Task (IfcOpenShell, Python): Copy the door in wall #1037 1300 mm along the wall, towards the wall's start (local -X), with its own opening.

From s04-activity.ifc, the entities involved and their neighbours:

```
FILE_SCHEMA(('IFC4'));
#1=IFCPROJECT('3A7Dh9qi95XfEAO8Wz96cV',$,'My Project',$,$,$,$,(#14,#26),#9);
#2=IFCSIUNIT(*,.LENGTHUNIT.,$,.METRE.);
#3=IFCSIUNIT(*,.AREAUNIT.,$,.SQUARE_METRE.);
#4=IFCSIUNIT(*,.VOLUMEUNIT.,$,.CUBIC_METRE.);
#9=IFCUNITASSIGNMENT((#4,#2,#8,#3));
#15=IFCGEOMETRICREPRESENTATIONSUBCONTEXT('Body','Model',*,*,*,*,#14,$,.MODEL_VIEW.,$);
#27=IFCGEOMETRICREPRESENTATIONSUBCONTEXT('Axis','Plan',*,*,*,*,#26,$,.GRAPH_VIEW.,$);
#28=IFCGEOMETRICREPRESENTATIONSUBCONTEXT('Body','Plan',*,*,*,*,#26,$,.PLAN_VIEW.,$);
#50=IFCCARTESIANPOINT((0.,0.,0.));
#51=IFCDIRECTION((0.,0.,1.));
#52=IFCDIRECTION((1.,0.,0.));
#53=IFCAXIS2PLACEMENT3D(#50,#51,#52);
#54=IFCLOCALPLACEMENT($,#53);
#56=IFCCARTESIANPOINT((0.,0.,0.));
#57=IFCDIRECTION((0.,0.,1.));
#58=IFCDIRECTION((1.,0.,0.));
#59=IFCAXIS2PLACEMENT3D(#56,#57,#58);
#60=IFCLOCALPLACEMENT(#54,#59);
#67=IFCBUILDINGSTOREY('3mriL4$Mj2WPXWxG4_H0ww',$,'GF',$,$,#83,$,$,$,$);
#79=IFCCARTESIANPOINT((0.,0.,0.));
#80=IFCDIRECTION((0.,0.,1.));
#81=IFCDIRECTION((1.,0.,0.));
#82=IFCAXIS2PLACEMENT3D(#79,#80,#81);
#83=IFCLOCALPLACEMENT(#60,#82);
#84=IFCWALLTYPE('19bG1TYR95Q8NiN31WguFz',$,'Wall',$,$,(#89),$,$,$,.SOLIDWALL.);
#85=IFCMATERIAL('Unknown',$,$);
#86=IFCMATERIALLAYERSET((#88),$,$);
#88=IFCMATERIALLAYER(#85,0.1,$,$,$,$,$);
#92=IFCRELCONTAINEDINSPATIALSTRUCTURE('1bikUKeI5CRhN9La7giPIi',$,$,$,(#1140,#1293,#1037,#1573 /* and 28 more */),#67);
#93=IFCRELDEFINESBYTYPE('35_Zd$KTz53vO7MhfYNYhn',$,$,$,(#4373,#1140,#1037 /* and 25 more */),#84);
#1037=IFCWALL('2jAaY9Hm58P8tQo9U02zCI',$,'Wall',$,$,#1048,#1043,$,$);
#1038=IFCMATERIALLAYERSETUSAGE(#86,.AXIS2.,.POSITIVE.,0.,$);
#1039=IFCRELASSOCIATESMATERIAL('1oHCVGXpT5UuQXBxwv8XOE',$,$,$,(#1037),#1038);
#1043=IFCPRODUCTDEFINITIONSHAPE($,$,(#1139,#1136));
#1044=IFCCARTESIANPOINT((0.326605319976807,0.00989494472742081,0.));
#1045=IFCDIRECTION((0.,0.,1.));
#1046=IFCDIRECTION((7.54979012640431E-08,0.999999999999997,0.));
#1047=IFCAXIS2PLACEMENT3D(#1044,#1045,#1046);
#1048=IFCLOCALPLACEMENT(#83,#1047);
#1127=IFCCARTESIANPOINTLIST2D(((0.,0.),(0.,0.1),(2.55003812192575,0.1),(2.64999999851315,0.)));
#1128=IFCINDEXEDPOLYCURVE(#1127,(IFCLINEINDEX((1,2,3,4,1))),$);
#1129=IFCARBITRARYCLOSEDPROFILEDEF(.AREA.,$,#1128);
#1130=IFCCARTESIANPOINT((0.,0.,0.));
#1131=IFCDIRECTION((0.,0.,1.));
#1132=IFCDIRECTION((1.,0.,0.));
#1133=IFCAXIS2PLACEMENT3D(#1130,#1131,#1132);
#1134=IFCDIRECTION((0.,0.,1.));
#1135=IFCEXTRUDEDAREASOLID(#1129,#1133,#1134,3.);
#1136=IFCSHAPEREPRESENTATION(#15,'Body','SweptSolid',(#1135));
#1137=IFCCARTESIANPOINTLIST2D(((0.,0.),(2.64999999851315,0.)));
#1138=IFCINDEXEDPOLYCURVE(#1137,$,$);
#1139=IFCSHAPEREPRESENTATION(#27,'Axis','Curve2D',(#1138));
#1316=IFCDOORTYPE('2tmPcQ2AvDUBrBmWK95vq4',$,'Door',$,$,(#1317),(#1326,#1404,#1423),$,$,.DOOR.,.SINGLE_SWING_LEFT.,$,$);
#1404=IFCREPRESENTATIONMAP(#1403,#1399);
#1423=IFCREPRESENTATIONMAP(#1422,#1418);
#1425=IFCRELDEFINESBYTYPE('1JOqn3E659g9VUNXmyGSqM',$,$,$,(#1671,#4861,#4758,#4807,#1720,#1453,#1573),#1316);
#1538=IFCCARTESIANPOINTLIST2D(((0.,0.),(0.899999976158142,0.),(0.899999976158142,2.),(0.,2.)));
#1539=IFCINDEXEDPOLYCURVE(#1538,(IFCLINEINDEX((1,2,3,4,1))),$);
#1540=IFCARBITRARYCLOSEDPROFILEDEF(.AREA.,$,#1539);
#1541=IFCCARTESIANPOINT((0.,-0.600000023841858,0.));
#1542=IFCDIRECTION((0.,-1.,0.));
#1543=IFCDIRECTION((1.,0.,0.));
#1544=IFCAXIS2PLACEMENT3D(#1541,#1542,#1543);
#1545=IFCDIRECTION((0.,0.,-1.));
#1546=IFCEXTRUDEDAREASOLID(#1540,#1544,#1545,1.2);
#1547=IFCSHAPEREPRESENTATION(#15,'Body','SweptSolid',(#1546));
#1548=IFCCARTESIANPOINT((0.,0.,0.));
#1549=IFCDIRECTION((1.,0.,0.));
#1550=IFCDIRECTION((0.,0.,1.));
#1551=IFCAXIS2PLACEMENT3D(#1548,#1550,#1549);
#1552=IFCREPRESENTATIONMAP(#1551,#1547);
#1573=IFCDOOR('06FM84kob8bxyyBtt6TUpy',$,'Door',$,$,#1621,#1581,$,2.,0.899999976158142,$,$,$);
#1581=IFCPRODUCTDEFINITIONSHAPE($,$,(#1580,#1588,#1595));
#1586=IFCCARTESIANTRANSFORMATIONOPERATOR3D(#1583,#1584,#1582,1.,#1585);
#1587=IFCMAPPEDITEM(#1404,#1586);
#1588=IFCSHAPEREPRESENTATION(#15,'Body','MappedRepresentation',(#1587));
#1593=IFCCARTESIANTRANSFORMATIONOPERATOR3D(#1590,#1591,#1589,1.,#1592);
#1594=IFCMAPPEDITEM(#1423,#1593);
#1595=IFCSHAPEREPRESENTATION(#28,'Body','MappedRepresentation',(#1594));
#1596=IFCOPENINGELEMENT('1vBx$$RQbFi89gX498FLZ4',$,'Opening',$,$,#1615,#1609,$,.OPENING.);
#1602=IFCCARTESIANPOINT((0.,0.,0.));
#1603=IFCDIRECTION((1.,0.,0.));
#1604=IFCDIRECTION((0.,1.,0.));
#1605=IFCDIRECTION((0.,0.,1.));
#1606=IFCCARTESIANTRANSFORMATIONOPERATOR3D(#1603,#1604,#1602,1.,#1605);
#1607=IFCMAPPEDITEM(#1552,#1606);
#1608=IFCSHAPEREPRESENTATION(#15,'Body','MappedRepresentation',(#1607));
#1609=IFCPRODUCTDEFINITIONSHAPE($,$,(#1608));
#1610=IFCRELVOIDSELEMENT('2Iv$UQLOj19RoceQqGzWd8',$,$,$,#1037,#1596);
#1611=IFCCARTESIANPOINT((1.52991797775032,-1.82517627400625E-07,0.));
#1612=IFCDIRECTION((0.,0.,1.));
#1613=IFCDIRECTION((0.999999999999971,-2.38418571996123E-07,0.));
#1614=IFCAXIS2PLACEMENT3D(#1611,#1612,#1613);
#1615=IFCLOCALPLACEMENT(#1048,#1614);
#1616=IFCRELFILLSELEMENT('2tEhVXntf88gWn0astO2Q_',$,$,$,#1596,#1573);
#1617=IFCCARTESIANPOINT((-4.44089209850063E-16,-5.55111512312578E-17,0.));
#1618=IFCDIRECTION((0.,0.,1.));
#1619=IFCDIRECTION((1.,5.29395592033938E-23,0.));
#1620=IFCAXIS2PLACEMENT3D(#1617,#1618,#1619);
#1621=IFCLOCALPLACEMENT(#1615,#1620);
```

```python
import ifcopenshell
import ifcopenshell.api.feature
import ifcopenshell.api.geometry
import ifcopenshell.api.root
import ifcopenshell.geom
import ifcopenshell.util.element
import ifcopenshell.util.placement
import ifcopenshell.util.shape

model = ifcopenshell.open("s04-activity.ifc")
settings = ifcopenshell.geom.settings()


def volume(element):
    """Net volume in cubic metres, openings subtracted."""
    shape = ifcopenshell.geom.create_shape(settings, element)
    return ifcopenshell.util.shape.get_volume(shape.geometry)


door = model.by_guid("06FM84kob8bxyyBtt6TUpy")
opening = door.FillsVoids[0].RelatingOpeningElement
wall = opening.VoidsElements[0].RelatingBuildingElement
before = volume(wall)
shift = ifcopenshell.util.placement.get_local_placement(wall.ObjectPlacement)[:3, 0] * -1.3

# copy_class copies the void relationship, type, container and properties, but no geometry.
new_opening = ifcopenshell.api.root.copy_class(model, product=opening)
new_opening.Representation = ifcopenshell.util.element.copy_deep(
    model, opening.Representation, exclude=["IfcGeometricRepresentationContext", "IfcRepresentationMap"]
)
new_door = ifcopenshell.api.root.copy_class(model, product=door)
new_door.Representation = ifcopenshell.util.element.copy_deep(
    model, door.Representation, exclude=["IfcGeometricRepresentationContext", "IfcRepresentationMap"]
)
ifcopenshell.api.feature.add_filling(model, opening=new_opening, element=new_door)

for old, new in ((opening, new_opening), (door, new_door)):
    matrix = ifcopenshell.util.placement.get_local_placement(old.ObjectPlacement)
    matrix[:3, 3] += shift
    ifcopenshell.api.geometry.edit_object_placement(model, product=new, matrix=matrix, is_si=False)

after = volume(wall)

print(f"wall volume {before:.3f} -> {after:.3f} m3")

model.write("s04-activity-out.ifc")
```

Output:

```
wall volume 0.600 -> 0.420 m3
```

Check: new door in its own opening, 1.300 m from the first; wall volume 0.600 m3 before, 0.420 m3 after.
